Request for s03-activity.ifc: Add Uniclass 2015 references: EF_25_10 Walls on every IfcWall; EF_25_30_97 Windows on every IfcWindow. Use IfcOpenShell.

First a look at what the model holds.

```python
import ifcopenshell

model = ifcopenshell.open("s03-activity.ifc")
print(model.schema)
print("classifications:", [c.Name for c in model.by_type("IfcClassification")])
for ifc_class in ("IfcDoor", "IfcRoof", "IfcStair", "IfcWall", "IfcWindow"):
    print(ifc_class, len(model.by_type(ifc_class)))
```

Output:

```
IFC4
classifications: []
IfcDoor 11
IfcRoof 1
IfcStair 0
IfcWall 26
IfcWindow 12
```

```python
import ifcopenshell
import ifcopenshell.api.classification

model = ifcopenshell.open("s03-activity.ifc")

system = ifcopenshell.api.classification.add_classification(model, classification="Uniclass 2015")

codes = {
    "IfcWall": ("EF_25_10", "Walls"),
    "IfcWindow": ("EF_25_30_97", "Windows"),
}
for ifc_class, (code, name) in codes.items():
    products = model.by_type(ifc_class)
    ifcopenshell.api.classification.add_reference(
        model, products=products, classification=system, identification=code, name=name
    )
    print(code, len(products))

model.write("s03-activity_rev.ifc")
```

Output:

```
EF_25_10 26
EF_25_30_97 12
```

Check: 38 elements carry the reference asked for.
